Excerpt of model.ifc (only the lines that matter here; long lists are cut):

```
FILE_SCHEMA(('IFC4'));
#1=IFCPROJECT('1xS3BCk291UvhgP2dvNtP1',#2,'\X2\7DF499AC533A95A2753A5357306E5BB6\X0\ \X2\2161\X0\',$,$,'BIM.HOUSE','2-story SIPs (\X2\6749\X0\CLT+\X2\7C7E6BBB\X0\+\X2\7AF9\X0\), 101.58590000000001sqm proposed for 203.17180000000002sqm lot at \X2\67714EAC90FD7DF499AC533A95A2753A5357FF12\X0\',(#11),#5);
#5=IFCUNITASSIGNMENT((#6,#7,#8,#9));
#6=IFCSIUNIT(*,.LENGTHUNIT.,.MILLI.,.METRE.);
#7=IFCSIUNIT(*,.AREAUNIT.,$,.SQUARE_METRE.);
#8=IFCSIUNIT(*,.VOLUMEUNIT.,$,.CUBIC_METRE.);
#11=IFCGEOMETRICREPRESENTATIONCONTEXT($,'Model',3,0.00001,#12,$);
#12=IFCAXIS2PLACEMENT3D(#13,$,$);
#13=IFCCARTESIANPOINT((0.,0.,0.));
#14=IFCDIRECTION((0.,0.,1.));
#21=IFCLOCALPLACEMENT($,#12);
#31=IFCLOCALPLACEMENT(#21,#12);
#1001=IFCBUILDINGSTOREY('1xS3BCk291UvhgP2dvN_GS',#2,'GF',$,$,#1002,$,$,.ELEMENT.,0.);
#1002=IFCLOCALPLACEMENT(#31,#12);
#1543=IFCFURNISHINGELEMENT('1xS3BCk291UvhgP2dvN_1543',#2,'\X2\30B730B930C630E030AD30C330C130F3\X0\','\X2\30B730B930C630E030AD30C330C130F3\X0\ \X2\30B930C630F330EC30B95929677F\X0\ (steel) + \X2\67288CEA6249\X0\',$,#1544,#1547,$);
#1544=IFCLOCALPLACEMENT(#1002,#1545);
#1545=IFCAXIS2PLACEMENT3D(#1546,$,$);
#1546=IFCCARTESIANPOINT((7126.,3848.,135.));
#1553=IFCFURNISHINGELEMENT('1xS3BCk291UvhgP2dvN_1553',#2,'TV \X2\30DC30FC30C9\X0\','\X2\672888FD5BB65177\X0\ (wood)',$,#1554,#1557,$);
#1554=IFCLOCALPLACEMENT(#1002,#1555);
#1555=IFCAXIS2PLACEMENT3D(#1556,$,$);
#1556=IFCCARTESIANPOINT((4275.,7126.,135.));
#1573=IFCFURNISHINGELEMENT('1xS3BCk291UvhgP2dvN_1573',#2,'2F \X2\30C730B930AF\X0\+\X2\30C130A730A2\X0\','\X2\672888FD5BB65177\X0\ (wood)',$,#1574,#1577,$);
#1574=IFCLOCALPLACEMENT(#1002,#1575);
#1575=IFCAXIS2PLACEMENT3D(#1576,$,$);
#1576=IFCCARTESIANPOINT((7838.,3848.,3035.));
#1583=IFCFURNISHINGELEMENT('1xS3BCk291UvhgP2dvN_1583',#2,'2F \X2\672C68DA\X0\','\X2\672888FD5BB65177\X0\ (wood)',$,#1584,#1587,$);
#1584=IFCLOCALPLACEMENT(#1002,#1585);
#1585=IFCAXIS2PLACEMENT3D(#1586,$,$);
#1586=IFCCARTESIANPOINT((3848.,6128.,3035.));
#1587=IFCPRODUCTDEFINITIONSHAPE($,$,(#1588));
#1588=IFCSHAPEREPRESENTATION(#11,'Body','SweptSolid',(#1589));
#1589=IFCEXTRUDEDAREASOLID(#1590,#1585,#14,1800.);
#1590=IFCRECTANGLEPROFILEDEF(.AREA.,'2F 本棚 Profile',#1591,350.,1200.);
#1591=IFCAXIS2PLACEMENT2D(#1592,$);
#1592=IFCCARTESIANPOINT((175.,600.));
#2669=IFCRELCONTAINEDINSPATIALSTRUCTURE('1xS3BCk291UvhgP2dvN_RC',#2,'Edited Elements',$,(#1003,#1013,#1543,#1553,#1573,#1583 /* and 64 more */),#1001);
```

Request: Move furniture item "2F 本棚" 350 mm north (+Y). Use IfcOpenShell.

```python
import ifcopenshell
import ifcopenshell.api.geometry
import ifcopenshell.util.placement

model = ifcopenshell.open("model.ifc")

item = model.by_id(1583)
matrix = ifcopenshell.util.placement.get_local_placement(item.ObjectPlacement)
matrix[1, 3] += 350.0
ifcopenshell.api.geometry.edit_object_placement(model, product=item, matrix=matrix, is_si=False)

print(ifcopenshell.util.placement.get_local_placement(item.ObjectPlacement).round(3) + 0.0)

model.write("model_edited.ifc")
```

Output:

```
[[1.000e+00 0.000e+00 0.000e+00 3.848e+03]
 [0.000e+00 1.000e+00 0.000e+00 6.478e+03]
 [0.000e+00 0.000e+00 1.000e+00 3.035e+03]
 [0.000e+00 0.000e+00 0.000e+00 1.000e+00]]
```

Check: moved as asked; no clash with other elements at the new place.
